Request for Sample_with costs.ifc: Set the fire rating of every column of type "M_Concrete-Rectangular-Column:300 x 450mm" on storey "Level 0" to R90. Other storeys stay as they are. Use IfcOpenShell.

First a look at what the model holds.

```python
import ifcopenshell
import ifcopenshell.util.element

model = ifcopenshell.open("Sample_with costs.ifc")
print(model.schema)
storey = next(s for s in model.by_type("IfcBuildingStorey") if s.Name == "Level 0")
columns = [e for e in ifcopenshell.util.element.get_decomposition(storey) if e.is_a("IfcColumn")]
seen = {}
for e in columns:
    element_type = ifcopenshell.util.element.get_type(e)
    key = (element_type.Name if element_type != e and element_type else None, ifcopenshell.util.element.get_pset(e, "Pset_ColumnCommon", "FireRating"))
    seen[key] = seen.get(key, 0) + 1
for (name, value), count in sorted(seen.items(), key=str):
    print(count, "x", name, "|", value)
```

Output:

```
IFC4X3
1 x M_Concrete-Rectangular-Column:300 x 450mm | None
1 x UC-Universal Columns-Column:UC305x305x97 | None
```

```python
import ifcopenshell
import ifcopenshell.api.pset
import ifcopenshell.util.element

model = ifcopenshell.open("Sample_with costs.ifc")

storey = next(s for s in model.by_type("IfcBuildingStorey") if s.Name == "Level 0")
columns = [e for e in ifcopenshell.util.element.get_decomposition(storey) if e.is_a("IfcColumn")]

count = 0
for e in columns:
    element_type = ifcopenshell.util.element.get_type(e)
    if element_type in (None, e) or element_type.Name != "M_Concrete-Rectangular-Column:300 x 450mm":
        continue
    # add_pset returns the element's existing set when there is one.
    pset = ifcopenshell.api.pset.add_pset(model, product=e, name="Pset_ColumnCommon")
    ifcopenshell.api.pset.edit_pset(model, pset=pset, properties={"FireRating": "R90"})
    count += 1

print(count, "columns updated")

model.write("Sample_with costs_updated.ifc")
```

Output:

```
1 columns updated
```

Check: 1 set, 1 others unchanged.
